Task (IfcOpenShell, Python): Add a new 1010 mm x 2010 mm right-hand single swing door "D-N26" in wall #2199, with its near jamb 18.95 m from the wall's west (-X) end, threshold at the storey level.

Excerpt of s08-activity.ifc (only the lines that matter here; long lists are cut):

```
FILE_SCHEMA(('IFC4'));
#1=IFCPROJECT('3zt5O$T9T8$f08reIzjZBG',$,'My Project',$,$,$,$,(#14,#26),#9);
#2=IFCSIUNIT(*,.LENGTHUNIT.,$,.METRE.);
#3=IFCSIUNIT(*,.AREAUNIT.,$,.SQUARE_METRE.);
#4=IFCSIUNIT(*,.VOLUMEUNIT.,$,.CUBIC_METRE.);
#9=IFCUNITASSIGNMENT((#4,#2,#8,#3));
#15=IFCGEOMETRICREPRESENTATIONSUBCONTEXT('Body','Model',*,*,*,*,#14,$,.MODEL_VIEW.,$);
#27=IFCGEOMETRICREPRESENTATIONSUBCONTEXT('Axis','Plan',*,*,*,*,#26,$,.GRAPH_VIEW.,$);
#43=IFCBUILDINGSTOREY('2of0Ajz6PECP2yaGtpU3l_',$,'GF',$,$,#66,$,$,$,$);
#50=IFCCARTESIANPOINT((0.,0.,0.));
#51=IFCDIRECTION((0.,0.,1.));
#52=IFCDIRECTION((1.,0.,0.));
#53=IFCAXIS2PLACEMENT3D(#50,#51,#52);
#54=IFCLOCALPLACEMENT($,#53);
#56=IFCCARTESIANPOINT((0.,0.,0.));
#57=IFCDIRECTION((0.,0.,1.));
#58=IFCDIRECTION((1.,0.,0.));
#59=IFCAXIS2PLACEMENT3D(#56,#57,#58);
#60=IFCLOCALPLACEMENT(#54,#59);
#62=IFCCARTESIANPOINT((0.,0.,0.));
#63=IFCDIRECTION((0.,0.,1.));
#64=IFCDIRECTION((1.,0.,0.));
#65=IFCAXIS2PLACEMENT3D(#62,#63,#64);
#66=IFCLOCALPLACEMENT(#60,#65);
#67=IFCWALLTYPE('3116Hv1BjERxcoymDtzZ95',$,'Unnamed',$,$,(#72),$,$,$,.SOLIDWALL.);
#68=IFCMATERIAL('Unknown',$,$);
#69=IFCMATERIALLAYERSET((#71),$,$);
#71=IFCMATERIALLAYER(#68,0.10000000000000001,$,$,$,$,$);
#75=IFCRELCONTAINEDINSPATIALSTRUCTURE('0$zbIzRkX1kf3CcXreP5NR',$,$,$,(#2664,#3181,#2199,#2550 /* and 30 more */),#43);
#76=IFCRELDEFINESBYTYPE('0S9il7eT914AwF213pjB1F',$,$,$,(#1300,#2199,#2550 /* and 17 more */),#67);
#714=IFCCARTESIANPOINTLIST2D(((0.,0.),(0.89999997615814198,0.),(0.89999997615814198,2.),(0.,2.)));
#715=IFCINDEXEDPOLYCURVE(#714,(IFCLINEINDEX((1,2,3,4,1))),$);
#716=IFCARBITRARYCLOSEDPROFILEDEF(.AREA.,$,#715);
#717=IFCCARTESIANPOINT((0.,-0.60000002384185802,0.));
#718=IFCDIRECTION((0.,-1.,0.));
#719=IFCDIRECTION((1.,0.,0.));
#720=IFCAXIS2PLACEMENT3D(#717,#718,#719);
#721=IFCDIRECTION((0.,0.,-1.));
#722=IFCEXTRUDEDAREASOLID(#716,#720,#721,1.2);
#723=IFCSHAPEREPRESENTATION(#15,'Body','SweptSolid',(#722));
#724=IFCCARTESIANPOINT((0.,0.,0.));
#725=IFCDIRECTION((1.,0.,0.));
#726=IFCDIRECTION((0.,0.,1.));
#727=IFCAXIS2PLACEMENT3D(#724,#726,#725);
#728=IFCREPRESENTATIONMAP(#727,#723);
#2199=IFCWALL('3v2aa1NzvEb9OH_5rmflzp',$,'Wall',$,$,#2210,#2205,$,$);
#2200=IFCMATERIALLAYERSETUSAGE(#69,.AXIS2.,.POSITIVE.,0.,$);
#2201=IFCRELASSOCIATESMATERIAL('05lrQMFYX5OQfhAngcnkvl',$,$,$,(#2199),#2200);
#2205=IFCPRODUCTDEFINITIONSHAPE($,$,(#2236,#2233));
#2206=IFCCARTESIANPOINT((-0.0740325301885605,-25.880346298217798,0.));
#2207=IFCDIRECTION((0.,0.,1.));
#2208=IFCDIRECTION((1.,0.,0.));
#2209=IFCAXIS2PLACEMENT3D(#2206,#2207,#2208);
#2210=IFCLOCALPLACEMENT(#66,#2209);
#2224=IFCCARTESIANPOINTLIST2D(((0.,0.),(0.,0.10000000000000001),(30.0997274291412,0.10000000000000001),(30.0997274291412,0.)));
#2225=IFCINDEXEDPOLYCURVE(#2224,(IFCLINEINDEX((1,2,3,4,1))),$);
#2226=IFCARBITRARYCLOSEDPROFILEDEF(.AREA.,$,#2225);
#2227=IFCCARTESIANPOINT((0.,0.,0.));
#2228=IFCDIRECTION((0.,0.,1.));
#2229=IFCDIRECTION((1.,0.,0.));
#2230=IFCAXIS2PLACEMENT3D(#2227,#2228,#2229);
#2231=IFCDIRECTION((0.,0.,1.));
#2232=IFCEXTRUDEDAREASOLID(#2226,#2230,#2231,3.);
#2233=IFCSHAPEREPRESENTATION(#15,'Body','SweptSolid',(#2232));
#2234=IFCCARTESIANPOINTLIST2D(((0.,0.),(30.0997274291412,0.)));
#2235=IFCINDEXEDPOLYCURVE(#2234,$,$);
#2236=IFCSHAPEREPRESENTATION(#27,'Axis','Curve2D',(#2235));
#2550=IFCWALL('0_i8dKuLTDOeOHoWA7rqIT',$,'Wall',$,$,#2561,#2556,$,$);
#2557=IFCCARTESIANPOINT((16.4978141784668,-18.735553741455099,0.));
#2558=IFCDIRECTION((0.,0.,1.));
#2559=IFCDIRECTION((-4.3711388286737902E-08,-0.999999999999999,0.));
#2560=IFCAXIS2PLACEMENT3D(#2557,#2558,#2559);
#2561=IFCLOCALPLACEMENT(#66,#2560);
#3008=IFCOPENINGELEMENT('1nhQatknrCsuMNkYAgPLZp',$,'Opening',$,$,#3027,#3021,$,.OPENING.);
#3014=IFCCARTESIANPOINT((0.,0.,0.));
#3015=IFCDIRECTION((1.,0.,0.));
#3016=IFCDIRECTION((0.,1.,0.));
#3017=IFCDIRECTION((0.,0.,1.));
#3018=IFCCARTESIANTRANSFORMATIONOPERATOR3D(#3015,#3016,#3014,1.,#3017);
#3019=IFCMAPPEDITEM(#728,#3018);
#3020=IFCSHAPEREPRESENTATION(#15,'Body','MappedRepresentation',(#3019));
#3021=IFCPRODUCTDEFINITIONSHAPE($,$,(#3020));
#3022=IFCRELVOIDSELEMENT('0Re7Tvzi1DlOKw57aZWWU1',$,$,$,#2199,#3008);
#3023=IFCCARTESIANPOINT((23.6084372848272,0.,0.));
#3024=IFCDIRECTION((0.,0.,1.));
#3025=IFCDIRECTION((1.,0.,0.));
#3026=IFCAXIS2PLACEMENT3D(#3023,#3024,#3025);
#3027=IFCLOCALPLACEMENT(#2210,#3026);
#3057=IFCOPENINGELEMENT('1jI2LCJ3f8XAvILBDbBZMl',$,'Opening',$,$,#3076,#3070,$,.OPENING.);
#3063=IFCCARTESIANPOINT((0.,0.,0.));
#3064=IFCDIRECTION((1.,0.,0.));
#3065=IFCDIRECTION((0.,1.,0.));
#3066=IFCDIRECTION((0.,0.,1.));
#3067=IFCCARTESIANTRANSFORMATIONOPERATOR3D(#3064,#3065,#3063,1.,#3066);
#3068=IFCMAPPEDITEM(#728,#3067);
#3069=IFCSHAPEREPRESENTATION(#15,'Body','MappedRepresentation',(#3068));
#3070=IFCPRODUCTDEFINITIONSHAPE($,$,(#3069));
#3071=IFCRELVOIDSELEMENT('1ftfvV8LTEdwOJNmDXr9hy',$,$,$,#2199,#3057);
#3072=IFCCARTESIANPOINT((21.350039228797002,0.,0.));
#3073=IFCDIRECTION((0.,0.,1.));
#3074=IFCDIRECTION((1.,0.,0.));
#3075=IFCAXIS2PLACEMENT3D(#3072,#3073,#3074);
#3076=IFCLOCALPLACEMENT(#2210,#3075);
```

```python
import numpy as np
import ifcopenshell
import ifcopenshell.api.feature
import ifcopenshell.api.geometry
import ifcopenshell.api.root
import ifcopenshell.api.spatial
import ifcopenshell.geom
import ifcopenshell.util.element
import ifcopenshell.util.placement
import ifcopenshell.util.representation
import ifcopenshell.util.shape
import ifcopenshell.util.unit

model = ifcopenshell.open("s08-activity.ifc")
unit_scale = ifcopenshell.util.unit.calculate_unit_scale(model)
settings = ifcopenshell.geom.settings()


def volume(element):
    """Net volume in cubic metres, openings subtracted."""
    shape = ifcopenshell.geom.create_shape(settings, element)
    return ifcopenshell.util.shape.get_volume(shape.geometry)


wall = model.by_id(2199)
storey = ifcopenshell.util.element.get_container(wall, ifc_class="IfcBuildingStorey")
context = ifcopenshell.util.representation.get_context(model, "Model", "Body", "MODEL_VIEW")
before = volume(wall)

width, height, from_end, sill = 1.01, 2.01, 18.95, 0.0  # metres

# The wall runs along its own X axis, and the end named is its -X end.
wall_shape = ifcopenshell.geom.create_shape(settings, wall)
x, y, z = ifcopenshell.util.shape.get_vertices(wall_shape.geometry).T
start = x.min() + from_end
face, thickness = float(y.min()), float(y.max() - y.min())
wall_matrix = ifcopenshell.util.placement.get_local_placement(wall.ObjectPlacement)
level = ifcopenshell.util.placement.get_local_placement(storey.ObjectPlacement)[2, 3]


def in_wall(x, y):
    """Placement at x, y metres in the wall's axes, at sill height."""
    matrix = wall_matrix.copy()
    matrix[:, 3] = wall_matrix @ np.array([x / unit_scale, y / unit_scale, 0.0, 1.0])
    matrix[2, 3] = level + sill / unit_scale
    return matrix


# Opening: a box that overshoots both wall faces by 50 mm.
opening = ifcopenshell.api.root.create_entity(model, ifc_class="IfcOpeningElement", predefined_type="OPENING")
box = ifcopenshell.api.geometry.add_wall_representation(
    model, context=context, length=width, height=height, thickness=thickness + 0.1
)
ifcopenshell.api.geometry.assign_representation(model, product=opening, representation=box)
ifcopenshell.api.geometry.edit_object_placement(model, product=opening, matrix=in_wall(start, face - 0.05), is_si=False)
ifcopenshell.api.feature.add_feature(model, feature=opening, element=wall)

door = ifcopenshell.api.root.create_entity(model, ifc_class="IfcDoor", name="D-N26", predefined_type="DOOR")
door.OverallWidth, door.OverallHeight = width / unit_scale, height / unit_scale
door.OperationType = "SINGLE_SWING_RIGHT"
body = ifcopenshell.api.geometry.add_door_representation(
    model,
    context=context,
    overall_width=door.OverallWidth,
    overall_height=door.OverallHeight,
    operation_type="SINGLE_SWING_RIGHT",
    lining_properties={"LiningDepth": thickness / unit_scale, "ThresholdDepth": thickness / unit_scale},
)
ifcopenshell.api.geometry.assign_representation(model, product=door, representation=body)
ifcopenshell.api.spatial.assign_container(model, products=[door], relating_structure=storey)
ifcopenshell.api.feature.add_filling(model, opening=opening, element=door)

# The lining spans the wall, so the door starts at the wall face.
ifcopenshell.api.geometry.edit_object_placement(model, product=door, matrix=in_wall(start, face), is_si=False)

after = volume(wall)

print(f"wall volume {before:.3f} -> {after:.3f} m3")

model.write("s08-activity_edited.ifc")
```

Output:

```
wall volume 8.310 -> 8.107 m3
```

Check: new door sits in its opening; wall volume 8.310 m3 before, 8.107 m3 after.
